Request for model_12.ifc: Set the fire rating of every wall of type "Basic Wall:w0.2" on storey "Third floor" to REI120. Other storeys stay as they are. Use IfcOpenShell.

First a look at what the model holds.

```python
import ifcopenshell
import ifcopenshell.util.element

model = ifcopenshell.open("model_12.ifc")
print(model.schema)
storey = next(s for s in model.by_type("IfcBuildingStorey") if s.Name == "Third floor")
walls = [e for e in ifcopenshell.util.element.get_decomposition(storey) if e.is_a("IfcWall")]
seen = {}
for e in walls:
    element_type = ifcopenshell.util.element.get_type(e)
    key = (element_type.Name if element_type != e and element_type else None, ifcopenshell.util.element.get_pset(e, "Pset_WallCommon", "FireRating"))
    seen[key] = seen.get(key, 0) + 1
for (name, value), count in sorted(seen.items(), key=str):
    print(count, "x", name, "|", value)
```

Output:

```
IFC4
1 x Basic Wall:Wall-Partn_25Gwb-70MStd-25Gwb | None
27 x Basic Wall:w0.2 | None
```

```python
import ifcopenshell
import ifcopenshell.api.pset
import ifcopenshell.util.element

model = ifcopenshell.open("model_12.ifc")

storey = next(s for s in model.by_type("IfcBuildingStorey") if s.Name == "Third floor")
walls = [e for e in ifcopenshell.util.element.get_decomposition(storey) if e.is_a("IfcWall")]

count = 0
for e in walls:
    element_type = ifcopenshell.util.element.get_type(e)
    if element_type in (None, e) or element_type.Name != "Basic Wall:w0.2":
        continue
    # add_pset returns the element's existing set when there is one.
    pset = ifcopenshell.api.pset.add_pset(model, product=e, name="Pset_WallCommon")
    ifcopenshell.api.pset.edit_pset(model, pset=pset, properties={"FireRating": "REI120"})
    count += 1

print(count, "walls updated")

model.write("model_12_v2.ifc")
```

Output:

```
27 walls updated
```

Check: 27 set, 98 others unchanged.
